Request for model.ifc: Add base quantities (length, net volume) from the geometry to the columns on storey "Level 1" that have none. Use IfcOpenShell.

First a look at what the model holds.

```python
import ifcopenshell
import ifcopenshell.util.element
import ifcopenshell.util.unit

model = ifcopenshell.open("model.ifc")
print(model.schema)
for unit_type in ("LENGTHUNIT", "AREAUNIT", "VOLUMEUNIT"):
    print(unit_type, ifcopenshell.util.unit.calculate_unit_scale(model, unit_type))
storey = next(s for s in model.by_type("IfcBuildingStorey") if s.Name == "Level 1")
columns = [e for e in ifcopenshell.util.element.get_decomposition(storey) if e.is_a("IfcColumn")]
for e in sorted(columns, key=lambda e: e.id()):
    print(e.id(), e.is_a(), e.Name, list(ifcopenshell.util.element.get_psets(e, qtos_only=True)), sep=" | ")
```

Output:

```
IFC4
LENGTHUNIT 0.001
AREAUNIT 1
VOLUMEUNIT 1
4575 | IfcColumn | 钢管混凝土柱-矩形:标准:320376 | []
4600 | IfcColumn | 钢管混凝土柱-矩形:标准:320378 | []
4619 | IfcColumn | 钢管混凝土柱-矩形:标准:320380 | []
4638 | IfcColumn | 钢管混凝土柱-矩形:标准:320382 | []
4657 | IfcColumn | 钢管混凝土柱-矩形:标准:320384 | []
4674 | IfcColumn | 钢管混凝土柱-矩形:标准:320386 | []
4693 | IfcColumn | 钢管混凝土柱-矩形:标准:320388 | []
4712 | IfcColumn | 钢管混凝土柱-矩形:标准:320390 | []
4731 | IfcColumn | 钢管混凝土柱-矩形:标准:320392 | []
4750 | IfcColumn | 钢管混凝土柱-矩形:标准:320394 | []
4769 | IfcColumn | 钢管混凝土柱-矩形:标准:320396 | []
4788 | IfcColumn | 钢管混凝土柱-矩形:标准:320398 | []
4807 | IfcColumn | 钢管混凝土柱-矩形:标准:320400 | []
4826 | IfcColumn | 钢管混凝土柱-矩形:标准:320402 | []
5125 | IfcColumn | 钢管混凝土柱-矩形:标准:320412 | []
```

```python
import ifcopenshell
import ifcopenshell.api.pset
import ifcopenshell.geom
import ifcopenshell.util.element
import ifcopenshell.util.shape
import ifcopenshell.util.unit

model = ifcopenshell.open("model.ifc")
unit_scale = ifcopenshell.util.unit.calculate_unit_scale(model)
volume_scale = ifcopenshell.util.unit.calculate_unit_scale(model, "VOLUMEUNIT")
settings = ifcopenshell.geom.settings()

storey = next(s for s in model.by_type("IfcBuildingStorey") if s.Name == "Level 1")
columns = [e for e in ifcopenshell.util.element.get_decomposition(storey) if e.is_a("IfcColumn")]

for e in sorted(columns, key=lambda e: e.id()):
    if ifcopenshell.util.element.get_psets(e, qtos_only=True, should_inherit=False):
        continue
    # Geometry comes back in metres, in the element's own axes.
    shape = ifcopenshell.geom.create_shape(settings, e)
    values = {
        "Length": ifcopenshell.util.shape.get_z(shape.geometry) / unit_scale,
        "NetVolume": ifcopenshell.util.shape.get_volume(shape.geometry) / volume_scale,
    }
    qto = ifcopenshell.api.pset.add_qto(model, product=e, name="Qto_ColumnBaseQuantities")
    ifcopenshell.api.pset.edit_qto(model, qto=qto, properties=values)
    print(e.id(), {k: round(v, 3) for k, v in values.items()})

model.write("model_edited.ifc")
```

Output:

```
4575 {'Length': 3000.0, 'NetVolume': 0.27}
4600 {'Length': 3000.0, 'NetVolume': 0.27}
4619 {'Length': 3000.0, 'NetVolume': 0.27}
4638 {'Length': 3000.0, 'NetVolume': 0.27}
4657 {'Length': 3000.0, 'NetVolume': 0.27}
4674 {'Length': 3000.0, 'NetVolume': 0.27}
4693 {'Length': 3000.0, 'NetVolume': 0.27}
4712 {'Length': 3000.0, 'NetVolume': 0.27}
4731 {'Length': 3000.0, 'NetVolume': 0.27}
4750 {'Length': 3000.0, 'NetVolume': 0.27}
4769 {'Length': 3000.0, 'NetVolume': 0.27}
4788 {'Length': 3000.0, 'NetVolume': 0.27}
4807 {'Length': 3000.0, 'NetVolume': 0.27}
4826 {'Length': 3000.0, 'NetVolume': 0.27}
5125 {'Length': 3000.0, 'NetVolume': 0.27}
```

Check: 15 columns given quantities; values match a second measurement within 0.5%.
